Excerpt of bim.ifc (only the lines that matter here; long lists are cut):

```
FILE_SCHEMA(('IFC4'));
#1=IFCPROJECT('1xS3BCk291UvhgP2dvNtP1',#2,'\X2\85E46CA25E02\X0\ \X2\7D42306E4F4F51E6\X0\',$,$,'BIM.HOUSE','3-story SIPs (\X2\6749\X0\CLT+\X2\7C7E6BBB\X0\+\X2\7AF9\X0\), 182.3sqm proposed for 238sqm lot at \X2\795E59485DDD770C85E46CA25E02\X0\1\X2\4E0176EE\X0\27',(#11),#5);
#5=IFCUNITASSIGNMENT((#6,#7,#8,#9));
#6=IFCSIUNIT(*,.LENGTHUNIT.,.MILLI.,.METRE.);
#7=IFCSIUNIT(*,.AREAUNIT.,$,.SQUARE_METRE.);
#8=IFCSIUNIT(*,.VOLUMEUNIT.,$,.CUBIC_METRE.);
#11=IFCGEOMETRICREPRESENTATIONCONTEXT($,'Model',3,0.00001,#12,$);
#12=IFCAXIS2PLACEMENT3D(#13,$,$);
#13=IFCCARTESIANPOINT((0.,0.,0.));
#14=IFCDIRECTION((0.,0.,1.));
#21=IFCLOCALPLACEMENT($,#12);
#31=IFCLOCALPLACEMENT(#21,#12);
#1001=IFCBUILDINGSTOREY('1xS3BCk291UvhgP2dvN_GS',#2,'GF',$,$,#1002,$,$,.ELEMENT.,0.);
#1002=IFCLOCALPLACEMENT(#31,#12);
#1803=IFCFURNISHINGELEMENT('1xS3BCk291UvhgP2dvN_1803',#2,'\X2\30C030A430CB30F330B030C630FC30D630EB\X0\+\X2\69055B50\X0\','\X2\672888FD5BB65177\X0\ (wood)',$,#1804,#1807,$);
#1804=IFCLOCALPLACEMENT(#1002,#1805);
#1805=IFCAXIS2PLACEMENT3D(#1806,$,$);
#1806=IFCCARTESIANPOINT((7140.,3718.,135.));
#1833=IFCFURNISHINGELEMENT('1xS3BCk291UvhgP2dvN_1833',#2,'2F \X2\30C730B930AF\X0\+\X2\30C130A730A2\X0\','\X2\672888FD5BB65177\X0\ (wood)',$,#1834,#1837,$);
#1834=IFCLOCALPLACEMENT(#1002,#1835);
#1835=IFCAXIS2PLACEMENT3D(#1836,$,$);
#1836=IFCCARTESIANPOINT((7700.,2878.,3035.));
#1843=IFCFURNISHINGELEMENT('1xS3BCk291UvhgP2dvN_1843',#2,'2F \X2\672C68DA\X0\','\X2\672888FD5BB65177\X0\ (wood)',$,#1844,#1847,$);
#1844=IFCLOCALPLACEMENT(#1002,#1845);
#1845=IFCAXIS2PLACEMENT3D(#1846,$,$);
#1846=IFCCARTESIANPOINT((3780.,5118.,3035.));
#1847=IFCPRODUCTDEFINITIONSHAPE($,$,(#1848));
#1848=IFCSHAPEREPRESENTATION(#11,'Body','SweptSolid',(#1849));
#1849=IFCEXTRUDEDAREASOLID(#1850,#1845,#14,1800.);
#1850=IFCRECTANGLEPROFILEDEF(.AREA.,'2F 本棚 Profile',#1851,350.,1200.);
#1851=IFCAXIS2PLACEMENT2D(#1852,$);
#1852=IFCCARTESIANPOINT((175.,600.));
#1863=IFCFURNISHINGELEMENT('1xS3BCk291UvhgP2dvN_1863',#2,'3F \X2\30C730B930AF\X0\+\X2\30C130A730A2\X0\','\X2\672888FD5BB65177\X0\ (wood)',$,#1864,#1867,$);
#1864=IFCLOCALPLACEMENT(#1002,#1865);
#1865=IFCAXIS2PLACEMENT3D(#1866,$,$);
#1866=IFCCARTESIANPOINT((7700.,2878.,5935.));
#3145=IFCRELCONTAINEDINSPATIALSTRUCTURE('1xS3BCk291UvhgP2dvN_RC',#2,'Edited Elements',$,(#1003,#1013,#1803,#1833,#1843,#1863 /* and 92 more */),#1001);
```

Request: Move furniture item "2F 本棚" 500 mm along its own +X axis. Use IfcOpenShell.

```python
import ifcopenshell
import ifcopenshell.api.geometry
import ifcopenshell.util.placement

model = ifcopenshell.open("bim.ifc")

item = model.by_id(1843)
matrix = ifcopenshell.util.placement.get_local_placement(item.ObjectPlacement)
matrix[:3, 3] += matrix[:3, 0] * 500.0
ifcopenshell.api.geometry.edit_object_placement(model, product=item, matrix=matrix, is_si=False)

print(ifcopenshell.util.placement.get_local_placement(item.ObjectPlacement).round(3) + 0.0)

model.write("bim_edited.ifc")
```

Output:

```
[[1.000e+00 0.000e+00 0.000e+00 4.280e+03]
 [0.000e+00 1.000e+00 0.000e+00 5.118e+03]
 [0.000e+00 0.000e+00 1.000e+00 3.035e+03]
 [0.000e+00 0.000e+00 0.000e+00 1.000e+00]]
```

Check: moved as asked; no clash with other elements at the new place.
